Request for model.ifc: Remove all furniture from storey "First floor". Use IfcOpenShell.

First a look at what the model holds.

```python
import ifcopenshell
import ifcopenshell.util.element

model = ifcopenshell.open("model.ifc")
print(model.schema)
storey = next(s for s in model.by_type("IfcBuildingStorey") if s.Name == "First floor")
furniture = [e for e in ifcopenshell.util.element.get_decomposition(storey) if e.is_a("IfcFurnishingElement")]
seen = {}
for e in furniture:
    element_type = ifcopenshell.util.element.get_type(e)
    name = element_type.Name if element_type not in (None, e) else None
    seen[name] = seen.get(name, 0) + 1
for name, count in sorted(seen.items(), key=str):
    print(count, "x", name)
```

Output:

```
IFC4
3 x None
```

```python
import ifcopenshell
import ifcopenshell.api.root
import ifcopenshell.util.element

model = ifcopenshell.open("model.ifc")

storey = next(s for s in model.by_type("IfcBuildingStorey") if s.Name == "First floor")
furniture = [e for e in ifcopenshell.util.element.get_decomposition(storey) if e.is_a("IfcFurnishingElement")]

for e in furniture:
    ifcopenshell.api.root.remove_product(model, product=e)
print(len(furniture), "removed")

model.write("model_v2.ifc")
```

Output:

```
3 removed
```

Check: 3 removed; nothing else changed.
